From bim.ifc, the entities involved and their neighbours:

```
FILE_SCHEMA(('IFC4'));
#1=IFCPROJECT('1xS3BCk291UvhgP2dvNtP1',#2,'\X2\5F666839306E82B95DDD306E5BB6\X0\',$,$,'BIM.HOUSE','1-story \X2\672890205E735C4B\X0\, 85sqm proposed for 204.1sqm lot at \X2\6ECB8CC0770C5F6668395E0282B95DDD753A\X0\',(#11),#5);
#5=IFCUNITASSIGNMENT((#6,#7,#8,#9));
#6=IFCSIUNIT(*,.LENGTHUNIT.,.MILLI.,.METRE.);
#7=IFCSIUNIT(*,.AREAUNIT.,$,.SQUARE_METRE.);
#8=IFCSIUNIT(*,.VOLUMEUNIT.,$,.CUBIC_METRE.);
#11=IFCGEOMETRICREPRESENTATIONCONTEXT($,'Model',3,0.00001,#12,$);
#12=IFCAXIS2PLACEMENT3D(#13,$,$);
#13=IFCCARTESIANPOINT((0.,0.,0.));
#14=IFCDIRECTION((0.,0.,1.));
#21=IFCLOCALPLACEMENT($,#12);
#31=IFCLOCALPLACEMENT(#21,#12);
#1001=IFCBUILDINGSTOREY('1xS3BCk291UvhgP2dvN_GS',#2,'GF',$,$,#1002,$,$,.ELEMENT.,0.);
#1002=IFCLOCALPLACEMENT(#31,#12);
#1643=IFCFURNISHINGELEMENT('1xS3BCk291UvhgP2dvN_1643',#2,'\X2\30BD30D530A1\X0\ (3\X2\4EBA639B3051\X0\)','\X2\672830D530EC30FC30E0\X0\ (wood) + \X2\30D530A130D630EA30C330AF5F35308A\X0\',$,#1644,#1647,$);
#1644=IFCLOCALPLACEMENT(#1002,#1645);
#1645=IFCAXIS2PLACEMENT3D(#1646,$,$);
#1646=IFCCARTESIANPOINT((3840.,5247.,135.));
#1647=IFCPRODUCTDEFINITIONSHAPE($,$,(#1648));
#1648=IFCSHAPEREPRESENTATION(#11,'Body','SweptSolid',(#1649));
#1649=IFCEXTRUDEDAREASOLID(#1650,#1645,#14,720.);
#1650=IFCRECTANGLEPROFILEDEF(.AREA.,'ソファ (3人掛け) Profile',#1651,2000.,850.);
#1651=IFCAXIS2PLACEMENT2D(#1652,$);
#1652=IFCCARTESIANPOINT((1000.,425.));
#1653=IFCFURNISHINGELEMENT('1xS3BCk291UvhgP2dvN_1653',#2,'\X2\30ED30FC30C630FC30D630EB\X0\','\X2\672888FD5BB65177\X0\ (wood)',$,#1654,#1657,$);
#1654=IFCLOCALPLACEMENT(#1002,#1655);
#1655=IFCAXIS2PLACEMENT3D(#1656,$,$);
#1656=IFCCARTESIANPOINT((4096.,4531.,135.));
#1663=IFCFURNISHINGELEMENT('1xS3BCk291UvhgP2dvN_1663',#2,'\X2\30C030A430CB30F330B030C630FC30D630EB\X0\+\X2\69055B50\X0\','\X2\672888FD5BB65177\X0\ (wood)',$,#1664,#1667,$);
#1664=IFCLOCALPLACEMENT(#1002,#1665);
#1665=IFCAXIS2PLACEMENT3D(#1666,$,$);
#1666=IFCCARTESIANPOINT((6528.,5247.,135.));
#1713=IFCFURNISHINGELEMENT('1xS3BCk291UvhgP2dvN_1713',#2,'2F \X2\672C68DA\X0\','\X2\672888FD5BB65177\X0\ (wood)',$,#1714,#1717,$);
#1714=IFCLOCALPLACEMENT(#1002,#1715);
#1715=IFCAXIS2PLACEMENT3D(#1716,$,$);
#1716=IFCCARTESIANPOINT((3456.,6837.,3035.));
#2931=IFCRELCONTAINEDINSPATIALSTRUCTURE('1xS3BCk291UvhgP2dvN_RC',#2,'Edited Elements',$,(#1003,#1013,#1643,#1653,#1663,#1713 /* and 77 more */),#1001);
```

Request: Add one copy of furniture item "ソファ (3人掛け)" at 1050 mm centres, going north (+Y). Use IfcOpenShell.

```python
import numpy as np
import ifcopenshell
import ifcopenshell.api.geometry
import ifcopenshell.api.root
import ifcopenshell.util.element
import ifcopenshell.util.placement
import ifcopenshell.util.unit

model = ifcopenshell.open("bim.ifc")
unit_scale = ifcopenshell.util.unit.calculate_unit_scale(model)


def reuse_history(source, copy):
    """copy_class also copies each property set's owner history, people and application; keep the originals."""
    for rel in copy.IsDefinedBy:
        if rel.is_a("IfcRelDefinesByProperties") and (history := rel.RelatingPropertyDefinition.OwnerHistory):
            rel.RelatingPropertyDefinition.OwnerHistory = source.OwnerHistory
            ifcopenshell.util.element.remove_deep2(model, history)


source = model.by_guid("1xS3BCk291UvhgP2dvN_1643")
base = ifcopenshell.util.placement.get_local_placement(source.ObjectPlacement)
step = np.array([0.0, 1.0, 0.0]) * 1.05 / unit_scale

for i in range(1, 2):
    copy = ifcopenshell.api.root.copy_class(model, product=source)
    copy.Representation = ifcopenshell.util.element.copy_deep(
        model, source.Representation, exclude=["IfcGeometricRepresentationContext", "IfcRepresentationMap"]
    )
    reuse_history(source, copy)
    matrix = base.copy()
    matrix[:3, 3] += i * step
    print("added at", matrix[:3, 3].round(3) + 0.0)
    ifcopenshell.api.geometry.edit_object_placement(model, product=copy, matrix=matrix, is_si=False)

model.write("bim_rev.ifc")
```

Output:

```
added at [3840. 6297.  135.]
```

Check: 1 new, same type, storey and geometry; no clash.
